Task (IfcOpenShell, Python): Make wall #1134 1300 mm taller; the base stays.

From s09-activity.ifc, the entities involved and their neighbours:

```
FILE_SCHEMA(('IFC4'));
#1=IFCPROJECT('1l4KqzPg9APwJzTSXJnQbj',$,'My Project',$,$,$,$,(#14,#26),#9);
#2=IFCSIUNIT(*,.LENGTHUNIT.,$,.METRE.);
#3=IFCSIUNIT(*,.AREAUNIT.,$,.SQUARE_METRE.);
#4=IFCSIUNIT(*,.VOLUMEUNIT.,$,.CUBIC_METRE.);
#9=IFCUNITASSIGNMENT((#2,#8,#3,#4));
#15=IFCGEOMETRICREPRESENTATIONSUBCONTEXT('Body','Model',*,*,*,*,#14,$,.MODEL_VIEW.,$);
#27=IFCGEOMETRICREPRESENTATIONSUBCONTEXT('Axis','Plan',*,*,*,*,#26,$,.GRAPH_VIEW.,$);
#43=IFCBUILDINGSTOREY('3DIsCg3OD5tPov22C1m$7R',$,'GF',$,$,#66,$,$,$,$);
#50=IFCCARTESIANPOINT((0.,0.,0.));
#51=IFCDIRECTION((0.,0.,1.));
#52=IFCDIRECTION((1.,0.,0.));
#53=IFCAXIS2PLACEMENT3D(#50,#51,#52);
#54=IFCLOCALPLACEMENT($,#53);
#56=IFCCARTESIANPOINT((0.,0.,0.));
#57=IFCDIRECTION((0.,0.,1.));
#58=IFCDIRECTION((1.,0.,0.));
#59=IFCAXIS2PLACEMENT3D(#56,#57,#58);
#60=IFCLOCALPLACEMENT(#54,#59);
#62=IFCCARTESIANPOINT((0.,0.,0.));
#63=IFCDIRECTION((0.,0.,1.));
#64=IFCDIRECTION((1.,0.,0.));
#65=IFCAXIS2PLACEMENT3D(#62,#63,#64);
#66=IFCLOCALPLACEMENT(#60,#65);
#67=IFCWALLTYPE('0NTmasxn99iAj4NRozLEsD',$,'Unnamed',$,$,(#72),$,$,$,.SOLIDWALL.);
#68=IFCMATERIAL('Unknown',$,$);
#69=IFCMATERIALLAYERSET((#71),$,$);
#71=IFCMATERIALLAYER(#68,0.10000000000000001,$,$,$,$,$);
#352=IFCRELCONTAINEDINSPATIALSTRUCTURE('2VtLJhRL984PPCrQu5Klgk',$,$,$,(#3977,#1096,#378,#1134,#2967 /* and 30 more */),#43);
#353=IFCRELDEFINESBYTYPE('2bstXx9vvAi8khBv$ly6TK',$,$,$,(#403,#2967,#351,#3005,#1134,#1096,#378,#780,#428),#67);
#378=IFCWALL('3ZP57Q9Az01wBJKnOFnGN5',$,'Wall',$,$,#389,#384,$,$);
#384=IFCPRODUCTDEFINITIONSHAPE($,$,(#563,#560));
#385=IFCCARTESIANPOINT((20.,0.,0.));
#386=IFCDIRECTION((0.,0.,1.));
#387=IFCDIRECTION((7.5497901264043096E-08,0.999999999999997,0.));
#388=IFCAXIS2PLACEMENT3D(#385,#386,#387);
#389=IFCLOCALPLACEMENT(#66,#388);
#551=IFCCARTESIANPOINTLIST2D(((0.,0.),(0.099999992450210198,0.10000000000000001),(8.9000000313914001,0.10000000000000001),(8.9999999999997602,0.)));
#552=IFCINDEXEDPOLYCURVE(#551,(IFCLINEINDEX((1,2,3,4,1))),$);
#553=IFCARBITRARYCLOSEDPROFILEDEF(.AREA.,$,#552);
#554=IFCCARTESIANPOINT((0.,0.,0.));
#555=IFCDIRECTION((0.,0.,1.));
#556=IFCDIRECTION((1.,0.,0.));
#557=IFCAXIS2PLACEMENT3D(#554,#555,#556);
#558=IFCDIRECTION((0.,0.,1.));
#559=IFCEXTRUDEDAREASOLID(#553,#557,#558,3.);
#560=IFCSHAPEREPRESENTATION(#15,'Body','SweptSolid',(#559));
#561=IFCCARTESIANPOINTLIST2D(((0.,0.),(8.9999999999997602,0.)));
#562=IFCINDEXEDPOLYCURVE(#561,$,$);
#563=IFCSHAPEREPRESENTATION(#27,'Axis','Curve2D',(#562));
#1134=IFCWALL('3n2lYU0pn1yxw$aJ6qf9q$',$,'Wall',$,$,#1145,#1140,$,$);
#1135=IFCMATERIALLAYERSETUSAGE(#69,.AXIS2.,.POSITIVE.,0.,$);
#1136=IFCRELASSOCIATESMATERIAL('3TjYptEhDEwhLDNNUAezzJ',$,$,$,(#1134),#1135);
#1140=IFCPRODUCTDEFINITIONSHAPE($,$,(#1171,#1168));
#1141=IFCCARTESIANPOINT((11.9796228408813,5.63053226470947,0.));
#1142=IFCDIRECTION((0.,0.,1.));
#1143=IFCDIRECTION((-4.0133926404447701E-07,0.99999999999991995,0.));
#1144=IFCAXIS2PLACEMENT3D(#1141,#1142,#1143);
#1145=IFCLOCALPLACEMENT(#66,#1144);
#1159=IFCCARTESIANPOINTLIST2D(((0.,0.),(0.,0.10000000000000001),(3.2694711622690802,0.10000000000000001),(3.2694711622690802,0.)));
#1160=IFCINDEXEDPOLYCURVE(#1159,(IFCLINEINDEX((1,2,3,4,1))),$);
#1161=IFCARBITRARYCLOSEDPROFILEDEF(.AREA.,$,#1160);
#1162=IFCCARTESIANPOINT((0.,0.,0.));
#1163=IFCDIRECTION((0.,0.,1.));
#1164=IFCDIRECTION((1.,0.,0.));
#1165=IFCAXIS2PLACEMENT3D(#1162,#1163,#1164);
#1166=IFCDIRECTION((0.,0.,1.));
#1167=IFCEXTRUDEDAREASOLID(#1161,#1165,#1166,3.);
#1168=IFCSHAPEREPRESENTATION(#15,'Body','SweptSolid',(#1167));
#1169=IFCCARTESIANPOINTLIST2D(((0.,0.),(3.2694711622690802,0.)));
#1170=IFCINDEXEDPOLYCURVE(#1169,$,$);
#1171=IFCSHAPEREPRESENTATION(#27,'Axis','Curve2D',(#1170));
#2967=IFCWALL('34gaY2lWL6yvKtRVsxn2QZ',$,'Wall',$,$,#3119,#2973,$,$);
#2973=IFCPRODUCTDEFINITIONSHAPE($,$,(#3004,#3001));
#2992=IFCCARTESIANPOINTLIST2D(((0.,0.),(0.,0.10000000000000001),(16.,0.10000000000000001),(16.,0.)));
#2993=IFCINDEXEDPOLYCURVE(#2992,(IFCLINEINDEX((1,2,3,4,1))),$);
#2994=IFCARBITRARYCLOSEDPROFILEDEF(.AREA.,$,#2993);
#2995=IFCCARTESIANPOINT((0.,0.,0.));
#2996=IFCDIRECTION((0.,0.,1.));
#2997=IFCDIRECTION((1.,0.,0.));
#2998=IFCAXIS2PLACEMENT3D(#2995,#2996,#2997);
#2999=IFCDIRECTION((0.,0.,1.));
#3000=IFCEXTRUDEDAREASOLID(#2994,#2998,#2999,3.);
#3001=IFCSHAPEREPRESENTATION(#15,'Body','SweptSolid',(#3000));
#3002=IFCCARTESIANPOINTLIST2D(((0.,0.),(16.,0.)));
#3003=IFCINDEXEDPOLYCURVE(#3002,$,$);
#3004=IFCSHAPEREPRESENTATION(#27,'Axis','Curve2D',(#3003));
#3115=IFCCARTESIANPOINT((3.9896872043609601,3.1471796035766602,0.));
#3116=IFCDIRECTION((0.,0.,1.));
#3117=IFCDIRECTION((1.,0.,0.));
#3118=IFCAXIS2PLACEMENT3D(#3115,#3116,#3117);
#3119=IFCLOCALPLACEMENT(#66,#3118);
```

```python
import ifcopenshell
import ifcopenshell.geom
import ifcopenshell.util.representation
import ifcopenshell.util.shape
import ifcopenshell.util.unit

model = ifcopenshell.open("s09-activity.ifc")
unit_scale = ifcopenshell.util.unit.calculate_unit_scale(model)
settings = ifcopenshell.geom.settings()


def volume(element):
    """Net volume in cubic metres, openings subtracted."""
    shape = ifcopenshell.geom.create_shape(settings, element)
    return ifcopenshell.util.shape.get_volume(shape.geometry)


wall = model.by_guid("3n2lYU0pn1yxw$aJ6qf9q$")
before = volume(wall)

body = ifcopenshell.util.representation.get_representation(wall, "Model", "Body")
solid = body.Items[0]
old_height = solid.Depth
solid.Depth += 1.3 / unit_scale
after = volume(wall)

print(f"height {old_height:g} -> {solid.Depth:g}, volume {before:.3f} -> {after:.3f} m3")

model.write("s09-activity_rev.ifc")
```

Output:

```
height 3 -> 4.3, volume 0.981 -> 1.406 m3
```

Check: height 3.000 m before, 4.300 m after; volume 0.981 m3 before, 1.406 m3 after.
